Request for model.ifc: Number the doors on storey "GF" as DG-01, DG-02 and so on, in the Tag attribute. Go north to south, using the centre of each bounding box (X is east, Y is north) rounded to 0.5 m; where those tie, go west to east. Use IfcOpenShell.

First a look at what the model holds.

```python
import ifcopenshell
import ifcopenshell.util.element
import ifcopenshell.util.placement

model = ifcopenshell.open("model.ifc")
print(model.schema)
storey = next(s for s in model.by_type("IfcBuildingStorey") if s.Name == "GF")
doors = [e for e in ifcopenshell.util.element.get_decomposition(storey) if e.is_a("IfcDoor")]
for e in sorted(doors, key=lambda e: e.id()):
    origin = ifcopenshell.util.placement.get_local_placement(e.ObjectPlacement)[:3, 3]
    print(e.id(), e.Tag, e.Name, origin.round(2) + 0.0, sep=" | ")
```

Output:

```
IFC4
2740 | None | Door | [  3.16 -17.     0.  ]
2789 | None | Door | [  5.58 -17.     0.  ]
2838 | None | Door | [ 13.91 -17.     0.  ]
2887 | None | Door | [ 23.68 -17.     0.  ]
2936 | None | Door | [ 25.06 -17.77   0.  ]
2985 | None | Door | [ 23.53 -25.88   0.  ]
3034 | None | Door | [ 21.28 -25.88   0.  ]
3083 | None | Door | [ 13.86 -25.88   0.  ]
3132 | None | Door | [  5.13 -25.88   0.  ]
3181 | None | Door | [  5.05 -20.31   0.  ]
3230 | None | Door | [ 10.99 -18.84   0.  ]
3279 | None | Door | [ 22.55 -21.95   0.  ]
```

```python
import ifcopenshell
import ifcopenshell.geom
import ifcopenshell.util.element
import ifcopenshell.util.shape

model = ifcopenshell.open("model.ifc")
settings = ifcopenshell.geom.settings()
settings.set("use-world-coords", True)


def centre(element):
    shape = ifcopenshell.geom.create_shape(settings, element)
    return ifcopenshell.util.shape.get_bbox_centroid(shape.geometry)


storey = next(s for s in model.by_type("IfcBuildingStorey") if s.Name == "GF")
doors = [e for e in ifcopenshell.util.element.get_decomposition(storey) if e.is_a("IfcDoor")]

# Insertion points can sit at a corner or the storey origin, so sort by the geometry (in metres).
centres = {e: centre(e) for e in doors}
doors.sort(key=lambda e: (-round(centres[e][1] / 0.5), centres[e][0]))

for i, e in enumerate(doors, start=1):
    number = f"DG-{i:02d}"
    e.Tag = number
    print(e.id(), number)

model.write("model_rev.ifc")
```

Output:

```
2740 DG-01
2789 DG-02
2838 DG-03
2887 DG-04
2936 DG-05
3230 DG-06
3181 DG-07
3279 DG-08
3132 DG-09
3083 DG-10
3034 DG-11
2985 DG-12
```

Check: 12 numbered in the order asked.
